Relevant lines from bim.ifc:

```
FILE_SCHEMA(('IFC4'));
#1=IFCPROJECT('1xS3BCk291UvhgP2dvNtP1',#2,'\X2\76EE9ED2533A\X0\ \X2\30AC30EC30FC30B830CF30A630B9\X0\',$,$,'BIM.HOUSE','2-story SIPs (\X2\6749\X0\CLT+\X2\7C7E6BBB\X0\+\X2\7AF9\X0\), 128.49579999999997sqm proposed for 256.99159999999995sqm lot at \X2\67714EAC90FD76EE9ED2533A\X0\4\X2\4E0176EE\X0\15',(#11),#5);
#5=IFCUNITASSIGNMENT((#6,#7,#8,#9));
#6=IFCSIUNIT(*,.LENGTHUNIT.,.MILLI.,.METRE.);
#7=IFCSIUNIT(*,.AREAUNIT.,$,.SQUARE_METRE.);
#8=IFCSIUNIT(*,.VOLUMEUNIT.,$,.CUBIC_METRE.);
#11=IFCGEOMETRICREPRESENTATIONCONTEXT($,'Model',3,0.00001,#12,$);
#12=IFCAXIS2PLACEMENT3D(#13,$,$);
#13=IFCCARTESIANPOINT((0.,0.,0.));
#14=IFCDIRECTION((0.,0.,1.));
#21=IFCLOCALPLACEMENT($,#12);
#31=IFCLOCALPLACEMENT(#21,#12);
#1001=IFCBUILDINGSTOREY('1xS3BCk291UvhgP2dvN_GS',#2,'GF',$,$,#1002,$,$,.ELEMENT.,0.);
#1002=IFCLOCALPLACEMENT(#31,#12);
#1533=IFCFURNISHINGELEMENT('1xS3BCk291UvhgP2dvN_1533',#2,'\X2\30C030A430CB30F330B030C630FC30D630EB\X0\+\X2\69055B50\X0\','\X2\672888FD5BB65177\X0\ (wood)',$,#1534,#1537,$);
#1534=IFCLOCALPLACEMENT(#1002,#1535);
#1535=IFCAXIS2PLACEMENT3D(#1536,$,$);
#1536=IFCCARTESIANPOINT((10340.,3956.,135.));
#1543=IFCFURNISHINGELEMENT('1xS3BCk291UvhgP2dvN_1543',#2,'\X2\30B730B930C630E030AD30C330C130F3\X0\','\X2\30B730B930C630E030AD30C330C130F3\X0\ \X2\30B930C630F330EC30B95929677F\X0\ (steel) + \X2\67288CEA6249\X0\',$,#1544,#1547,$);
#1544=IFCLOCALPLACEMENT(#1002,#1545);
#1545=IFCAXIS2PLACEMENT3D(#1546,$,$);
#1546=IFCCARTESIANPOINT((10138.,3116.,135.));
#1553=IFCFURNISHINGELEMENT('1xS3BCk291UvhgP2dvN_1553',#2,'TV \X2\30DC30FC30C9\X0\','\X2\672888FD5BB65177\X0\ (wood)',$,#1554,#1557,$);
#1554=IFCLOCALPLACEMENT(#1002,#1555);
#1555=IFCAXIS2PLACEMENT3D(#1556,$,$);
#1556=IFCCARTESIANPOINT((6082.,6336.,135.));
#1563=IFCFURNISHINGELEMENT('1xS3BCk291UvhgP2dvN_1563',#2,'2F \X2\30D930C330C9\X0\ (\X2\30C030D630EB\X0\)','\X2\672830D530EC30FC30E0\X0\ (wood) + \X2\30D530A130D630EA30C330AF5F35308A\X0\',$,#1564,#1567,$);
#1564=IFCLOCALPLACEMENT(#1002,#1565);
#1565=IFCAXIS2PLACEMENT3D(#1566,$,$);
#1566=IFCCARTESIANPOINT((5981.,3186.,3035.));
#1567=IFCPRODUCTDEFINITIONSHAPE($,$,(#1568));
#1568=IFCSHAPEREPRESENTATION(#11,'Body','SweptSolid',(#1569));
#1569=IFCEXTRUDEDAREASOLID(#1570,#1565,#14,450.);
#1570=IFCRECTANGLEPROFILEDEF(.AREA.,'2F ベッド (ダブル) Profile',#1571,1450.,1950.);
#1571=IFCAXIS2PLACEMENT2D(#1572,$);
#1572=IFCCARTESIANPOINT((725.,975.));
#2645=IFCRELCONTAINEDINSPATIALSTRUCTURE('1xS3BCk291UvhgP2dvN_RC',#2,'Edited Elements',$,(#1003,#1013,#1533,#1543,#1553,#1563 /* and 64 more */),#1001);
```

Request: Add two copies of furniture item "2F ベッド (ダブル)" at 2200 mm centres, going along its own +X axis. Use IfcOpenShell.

```python
import ifcopenshell
import ifcopenshell.api.geometry
import ifcopenshell.api.root
import ifcopenshell.util.element
import ifcopenshell.util.placement

model = ifcopenshell.open("bim.ifc")


def reuse_history(source, copy):
    """copy_class also copies each property set's owner history, people and application; keep the originals."""
    for rel in copy.IsDefinedBy:
        if rel.is_a("IfcRelDefinesByProperties") and (history := rel.RelatingPropertyDefinition.OwnerHistory):
            rel.RelatingPropertyDefinition.OwnerHistory = source.OwnerHistory
            ifcopenshell.util.element.remove_deep2(model, history)


source = model.by_guid("1xS3BCk291UvhgP2dvN_1563")
base = ifcopenshell.util.placement.get_local_placement(source.ObjectPlacement)
step = base[:3, 0] * 2200.0

for i in range(1, 3):
    copy = ifcopenshell.api.root.copy_class(model, product=source)
    copy.Representation = ifcopenshell.util.element.copy_deep(
        model, source.Representation, exclude=["IfcGeometricRepresentationContext", "IfcRepresentationMap"]
    )
    reuse_history(source, copy)
    matrix = base.copy()
    matrix[:3, 3] += i * step
    print("added at", matrix[:3, 3].round(3) + 0.0)
    ifcopenshell.api.geometry.edit_object_placement(model, product=copy, matrix=matrix, is_si=False)

model.write("bim-out.ifc")
```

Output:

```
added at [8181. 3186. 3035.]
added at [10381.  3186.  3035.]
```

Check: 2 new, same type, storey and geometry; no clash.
